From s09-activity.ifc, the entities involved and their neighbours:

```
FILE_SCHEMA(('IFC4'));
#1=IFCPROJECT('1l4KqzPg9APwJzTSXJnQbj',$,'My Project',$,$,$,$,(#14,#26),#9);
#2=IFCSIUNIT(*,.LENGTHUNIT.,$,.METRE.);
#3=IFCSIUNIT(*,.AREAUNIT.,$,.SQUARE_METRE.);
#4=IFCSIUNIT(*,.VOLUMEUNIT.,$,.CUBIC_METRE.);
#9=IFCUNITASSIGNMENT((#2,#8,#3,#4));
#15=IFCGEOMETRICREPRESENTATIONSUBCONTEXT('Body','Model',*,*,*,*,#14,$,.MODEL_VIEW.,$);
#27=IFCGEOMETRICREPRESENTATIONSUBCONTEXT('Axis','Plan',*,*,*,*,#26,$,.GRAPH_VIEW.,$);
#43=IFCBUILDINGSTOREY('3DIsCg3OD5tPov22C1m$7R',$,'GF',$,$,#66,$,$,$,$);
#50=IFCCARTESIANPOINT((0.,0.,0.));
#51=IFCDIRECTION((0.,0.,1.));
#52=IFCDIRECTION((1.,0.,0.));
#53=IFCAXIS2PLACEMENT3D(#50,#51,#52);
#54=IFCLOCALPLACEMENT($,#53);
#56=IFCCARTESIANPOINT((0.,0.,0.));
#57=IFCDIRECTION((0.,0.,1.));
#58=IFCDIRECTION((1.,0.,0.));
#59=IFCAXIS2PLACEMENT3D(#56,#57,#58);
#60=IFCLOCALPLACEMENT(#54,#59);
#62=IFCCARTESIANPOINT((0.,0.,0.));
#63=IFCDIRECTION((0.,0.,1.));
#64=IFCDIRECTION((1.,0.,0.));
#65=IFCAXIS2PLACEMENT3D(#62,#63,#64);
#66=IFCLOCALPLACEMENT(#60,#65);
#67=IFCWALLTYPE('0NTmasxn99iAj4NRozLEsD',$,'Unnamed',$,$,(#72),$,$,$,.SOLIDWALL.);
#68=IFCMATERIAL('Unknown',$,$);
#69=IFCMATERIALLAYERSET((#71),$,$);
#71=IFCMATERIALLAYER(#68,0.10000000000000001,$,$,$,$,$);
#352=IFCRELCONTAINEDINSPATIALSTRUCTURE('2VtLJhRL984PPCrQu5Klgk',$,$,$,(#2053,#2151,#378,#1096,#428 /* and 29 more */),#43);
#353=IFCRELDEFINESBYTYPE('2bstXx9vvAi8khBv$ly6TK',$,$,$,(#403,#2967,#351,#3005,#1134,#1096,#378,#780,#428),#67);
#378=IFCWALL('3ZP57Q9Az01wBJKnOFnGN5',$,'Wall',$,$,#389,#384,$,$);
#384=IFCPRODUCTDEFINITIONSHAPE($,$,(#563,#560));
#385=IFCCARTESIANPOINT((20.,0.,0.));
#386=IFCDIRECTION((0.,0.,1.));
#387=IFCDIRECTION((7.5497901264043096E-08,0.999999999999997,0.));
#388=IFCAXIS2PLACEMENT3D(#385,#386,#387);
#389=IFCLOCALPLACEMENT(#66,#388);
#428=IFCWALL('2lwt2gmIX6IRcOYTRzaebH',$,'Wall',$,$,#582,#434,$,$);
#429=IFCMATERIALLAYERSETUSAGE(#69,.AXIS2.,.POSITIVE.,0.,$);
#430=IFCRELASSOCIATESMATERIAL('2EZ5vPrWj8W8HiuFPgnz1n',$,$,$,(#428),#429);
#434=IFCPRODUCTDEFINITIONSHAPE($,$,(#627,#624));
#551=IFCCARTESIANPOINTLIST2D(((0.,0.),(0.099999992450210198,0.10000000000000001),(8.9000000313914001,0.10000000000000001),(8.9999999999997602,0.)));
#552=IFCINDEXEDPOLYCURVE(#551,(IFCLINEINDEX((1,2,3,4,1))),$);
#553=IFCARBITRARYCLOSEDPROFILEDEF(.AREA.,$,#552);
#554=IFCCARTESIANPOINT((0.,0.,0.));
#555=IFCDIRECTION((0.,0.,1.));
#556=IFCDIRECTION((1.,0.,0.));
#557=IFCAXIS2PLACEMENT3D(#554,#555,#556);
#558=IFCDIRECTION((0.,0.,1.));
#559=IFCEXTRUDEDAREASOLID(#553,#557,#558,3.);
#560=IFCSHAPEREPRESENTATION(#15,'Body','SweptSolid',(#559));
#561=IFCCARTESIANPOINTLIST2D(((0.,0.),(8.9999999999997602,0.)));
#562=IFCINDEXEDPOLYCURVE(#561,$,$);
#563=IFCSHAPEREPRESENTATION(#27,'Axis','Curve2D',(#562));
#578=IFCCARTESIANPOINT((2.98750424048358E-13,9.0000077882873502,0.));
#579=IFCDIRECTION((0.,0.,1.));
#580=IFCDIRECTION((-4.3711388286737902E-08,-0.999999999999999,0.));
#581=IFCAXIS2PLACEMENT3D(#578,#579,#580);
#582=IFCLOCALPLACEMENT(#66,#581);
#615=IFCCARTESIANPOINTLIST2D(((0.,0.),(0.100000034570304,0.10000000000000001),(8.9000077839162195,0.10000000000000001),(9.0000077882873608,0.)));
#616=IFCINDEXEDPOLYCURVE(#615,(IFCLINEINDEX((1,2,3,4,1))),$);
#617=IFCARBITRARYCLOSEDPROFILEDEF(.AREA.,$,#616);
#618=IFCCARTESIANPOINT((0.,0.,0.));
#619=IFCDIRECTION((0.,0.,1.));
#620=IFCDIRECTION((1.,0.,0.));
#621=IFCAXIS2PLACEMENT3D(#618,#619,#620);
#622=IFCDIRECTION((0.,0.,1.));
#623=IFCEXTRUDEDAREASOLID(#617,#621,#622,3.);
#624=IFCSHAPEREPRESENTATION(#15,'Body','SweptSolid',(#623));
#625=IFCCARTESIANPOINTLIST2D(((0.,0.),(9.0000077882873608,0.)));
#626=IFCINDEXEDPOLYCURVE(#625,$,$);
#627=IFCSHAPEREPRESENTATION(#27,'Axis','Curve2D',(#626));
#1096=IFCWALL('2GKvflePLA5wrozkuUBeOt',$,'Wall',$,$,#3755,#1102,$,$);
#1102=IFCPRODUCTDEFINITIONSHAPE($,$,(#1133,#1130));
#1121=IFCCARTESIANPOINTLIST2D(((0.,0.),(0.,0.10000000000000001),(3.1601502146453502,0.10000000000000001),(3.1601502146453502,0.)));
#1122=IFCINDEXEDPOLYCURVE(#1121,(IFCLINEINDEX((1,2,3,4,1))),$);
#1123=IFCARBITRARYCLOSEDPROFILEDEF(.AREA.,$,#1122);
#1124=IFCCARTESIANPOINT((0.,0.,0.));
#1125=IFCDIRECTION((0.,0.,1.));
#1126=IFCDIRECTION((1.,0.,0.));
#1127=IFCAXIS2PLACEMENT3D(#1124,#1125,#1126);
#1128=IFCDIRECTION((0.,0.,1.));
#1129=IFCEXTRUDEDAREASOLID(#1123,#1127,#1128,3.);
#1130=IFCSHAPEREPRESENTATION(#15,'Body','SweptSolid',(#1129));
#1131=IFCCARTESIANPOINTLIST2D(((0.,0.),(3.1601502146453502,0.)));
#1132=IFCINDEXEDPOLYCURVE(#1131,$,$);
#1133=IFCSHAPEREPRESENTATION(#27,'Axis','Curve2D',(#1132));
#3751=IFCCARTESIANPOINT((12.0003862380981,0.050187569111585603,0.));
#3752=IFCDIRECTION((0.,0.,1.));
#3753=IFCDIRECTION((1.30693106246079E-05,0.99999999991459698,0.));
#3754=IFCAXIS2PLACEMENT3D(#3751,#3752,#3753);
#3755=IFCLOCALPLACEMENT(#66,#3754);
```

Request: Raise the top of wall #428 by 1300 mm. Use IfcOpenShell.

```python
import ifcopenshell
import ifcopenshell.geom
import ifcopenshell.util.representation
import ifcopenshell.util.shape
import ifcopenshell.util.unit

model = ifcopenshell.open("s09-activity.ifc")
unit_scale = ifcopenshell.util.unit.calculate_unit_scale(model)
settings = ifcopenshell.geom.settings()


def volume(element):
    """Net volume in cubic metres, openings subtracted."""
    shape = ifcopenshell.geom.create_shape(settings, element)
    return ifcopenshell.util.shape.get_volume(shape.geometry)


wall = model.by_guid("2lwt2gmIX6IRcOYTRzaebH")
before = volume(wall)

body = ifcopenshell.util.representation.get_representation(wall, "Model", "Body")
solid = body.Items[0]
old_height = solid.Depth
solid.Depth += 1.3 / unit_scale
after = volume(wall)

print(f"height {old_height:g} -> {solid.Depth:g}, volume {before:.3f} -> {after:.3f} m3")

model.write("s09-activity_rev.ifc")
```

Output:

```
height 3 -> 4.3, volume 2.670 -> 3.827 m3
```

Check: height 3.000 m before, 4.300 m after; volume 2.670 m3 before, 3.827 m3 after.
